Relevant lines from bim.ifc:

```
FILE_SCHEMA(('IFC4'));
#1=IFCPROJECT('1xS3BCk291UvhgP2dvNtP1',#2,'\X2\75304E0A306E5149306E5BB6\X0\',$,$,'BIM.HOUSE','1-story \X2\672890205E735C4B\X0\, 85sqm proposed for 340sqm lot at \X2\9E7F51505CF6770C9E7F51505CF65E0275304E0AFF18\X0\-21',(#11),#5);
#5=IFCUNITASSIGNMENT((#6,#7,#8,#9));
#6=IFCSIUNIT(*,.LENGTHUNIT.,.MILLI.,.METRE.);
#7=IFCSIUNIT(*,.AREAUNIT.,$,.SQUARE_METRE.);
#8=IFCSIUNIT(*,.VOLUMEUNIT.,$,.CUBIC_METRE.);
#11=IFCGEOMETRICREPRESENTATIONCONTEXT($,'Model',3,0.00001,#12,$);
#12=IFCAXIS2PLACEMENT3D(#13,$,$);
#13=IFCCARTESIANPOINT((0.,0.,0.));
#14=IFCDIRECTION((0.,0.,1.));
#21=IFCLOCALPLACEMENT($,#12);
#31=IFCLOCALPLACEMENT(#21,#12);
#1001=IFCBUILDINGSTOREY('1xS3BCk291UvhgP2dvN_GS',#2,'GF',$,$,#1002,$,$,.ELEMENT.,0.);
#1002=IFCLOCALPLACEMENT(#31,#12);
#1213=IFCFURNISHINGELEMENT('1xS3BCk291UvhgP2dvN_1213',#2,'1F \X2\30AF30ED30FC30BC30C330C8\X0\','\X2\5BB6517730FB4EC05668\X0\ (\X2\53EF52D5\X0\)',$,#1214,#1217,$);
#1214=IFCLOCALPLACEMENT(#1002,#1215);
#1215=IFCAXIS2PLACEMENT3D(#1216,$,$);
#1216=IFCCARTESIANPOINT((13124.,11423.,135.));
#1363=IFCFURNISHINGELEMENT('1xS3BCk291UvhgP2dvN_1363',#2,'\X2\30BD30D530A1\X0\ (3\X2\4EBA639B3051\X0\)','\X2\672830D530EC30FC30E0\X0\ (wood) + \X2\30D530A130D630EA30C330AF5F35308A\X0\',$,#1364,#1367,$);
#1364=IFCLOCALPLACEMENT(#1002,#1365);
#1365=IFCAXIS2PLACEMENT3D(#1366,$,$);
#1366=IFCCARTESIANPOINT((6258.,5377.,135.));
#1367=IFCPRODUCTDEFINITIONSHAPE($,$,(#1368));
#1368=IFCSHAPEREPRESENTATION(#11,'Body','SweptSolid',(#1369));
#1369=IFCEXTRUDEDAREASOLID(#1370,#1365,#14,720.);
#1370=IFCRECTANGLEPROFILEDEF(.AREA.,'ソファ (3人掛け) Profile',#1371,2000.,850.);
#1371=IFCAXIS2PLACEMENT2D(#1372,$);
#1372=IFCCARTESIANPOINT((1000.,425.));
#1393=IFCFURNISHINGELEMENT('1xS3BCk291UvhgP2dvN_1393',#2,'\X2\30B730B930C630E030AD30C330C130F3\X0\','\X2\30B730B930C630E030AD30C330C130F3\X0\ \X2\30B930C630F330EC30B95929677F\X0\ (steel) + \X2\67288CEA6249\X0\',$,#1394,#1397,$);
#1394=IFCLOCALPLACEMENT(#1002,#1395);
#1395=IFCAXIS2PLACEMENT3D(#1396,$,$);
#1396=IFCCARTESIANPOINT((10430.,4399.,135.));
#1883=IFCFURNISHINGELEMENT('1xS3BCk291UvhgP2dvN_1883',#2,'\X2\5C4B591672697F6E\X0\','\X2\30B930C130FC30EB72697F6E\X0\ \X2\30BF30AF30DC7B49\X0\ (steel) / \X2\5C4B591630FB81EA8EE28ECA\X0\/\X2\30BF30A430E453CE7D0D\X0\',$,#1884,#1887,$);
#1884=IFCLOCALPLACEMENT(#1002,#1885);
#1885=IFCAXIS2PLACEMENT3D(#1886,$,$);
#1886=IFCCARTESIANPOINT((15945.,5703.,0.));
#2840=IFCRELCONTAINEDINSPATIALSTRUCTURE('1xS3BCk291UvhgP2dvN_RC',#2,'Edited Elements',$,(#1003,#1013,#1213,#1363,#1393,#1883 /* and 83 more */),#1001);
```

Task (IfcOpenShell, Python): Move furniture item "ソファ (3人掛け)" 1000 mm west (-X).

```python
import ifcopenshell
import ifcopenshell.api.geometry
import ifcopenshell.util.placement

model = ifcopenshell.open("bim.ifc")

item = model.by_guid("1xS3BCk291UvhgP2dvN_1363")
matrix = ifcopenshell.util.placement.get_local_placement(item.ObjectPlacement)
matrix[0, 3] -= 1000.0
ifcopenshell.api.geometry.edit_object_placement(model, product=item, matrix=matrix, is_si=False)

print(ifcopenshell.util.placement.get_local_placement(item.ObjectPlacement).round(3) + 0.0)

model.write("bim_rev.ifc")
```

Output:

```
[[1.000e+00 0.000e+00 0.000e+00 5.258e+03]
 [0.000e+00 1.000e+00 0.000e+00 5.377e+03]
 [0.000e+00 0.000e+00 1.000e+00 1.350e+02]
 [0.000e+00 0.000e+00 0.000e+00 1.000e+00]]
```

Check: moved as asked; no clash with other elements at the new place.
